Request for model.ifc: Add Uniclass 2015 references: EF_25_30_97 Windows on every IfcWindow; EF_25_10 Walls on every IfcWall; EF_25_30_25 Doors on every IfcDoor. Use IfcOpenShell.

First a look at what the model holds.

```python
import ifcopenshell

model = ifcopenshell.open("model.ifc")
print(model.schema)
print("classifications:", [c.Name for c in model.by_type("IfcClassification")])
for ifc_class in ("IfcDoor", "IfcRoof", "IfcStair", "IfcWall", "IfcWindow"):
    print(ifc_class, len(model.by_type(ifc_class)))
```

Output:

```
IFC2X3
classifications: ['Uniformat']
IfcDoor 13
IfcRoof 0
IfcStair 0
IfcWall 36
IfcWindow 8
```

```python
import ifcopenshell
import ifcopenshell.api.classification

model = ifcopenshell.open("model.ifc")

# IFC2X3 requires Source and Edition and has no link from the project to the system.
system = model.create_entity("IfcClassification", Source="NBS", Edition="2015", Name="Uniclass 2015")

codes = {
    "IfcWindow": ("EF_25_30_97", "Windows"),
    "IfcWall": ("EF_25_10", "Walls"),
    "IfcDoor": ("EF_25_30_25", "Doors"),
}
for ifc_class, (code, name) in codes.items():
    products = model.by_type(ifc_class)
    ifcopenshell.api.classification.add_reference(
        model, products=products, classification=system, identification=code, name=name
    )
    print(code, len(products))

model.write("model-out.ifc")
```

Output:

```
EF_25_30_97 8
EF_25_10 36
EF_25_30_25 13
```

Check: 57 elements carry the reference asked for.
